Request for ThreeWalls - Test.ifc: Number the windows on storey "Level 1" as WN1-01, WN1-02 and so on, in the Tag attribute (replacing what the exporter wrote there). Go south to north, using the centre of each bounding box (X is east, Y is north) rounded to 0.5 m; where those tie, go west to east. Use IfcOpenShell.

First a look at what the model holds.

```python
import ifcopenshell
import ifcopenshell.util.element
import ifcopenshell.util.placement

model = ifcopenshell.open("ThreeWalls - Test.ifc")
print(model.schema)
storey = next(s for s in model.by_type("IfcBuildingStorey") if s.Name == "Level 1")
windows = [e for e in ifcopenshell.util.element.get_decomposition(storey) if e.is_a("IfcWindow")]
for e in sorted(windows, key=lambda e: e.id()):
    origin = ifcopenshell.util.placement.get_local_placement(e.ObjectPlacement)[:3, 3]
    print(e.id(), e.Tag, e.Name, origin.round(2) + 0.0, sep=" | ")
```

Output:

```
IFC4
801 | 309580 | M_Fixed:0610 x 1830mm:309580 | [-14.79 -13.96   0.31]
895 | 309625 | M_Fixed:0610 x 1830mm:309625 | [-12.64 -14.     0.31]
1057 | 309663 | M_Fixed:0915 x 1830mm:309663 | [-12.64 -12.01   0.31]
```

```python
import ifcopenshell
import ifcopenshell.geom
import ifcopenshell.util.element
import ifcopenshell.util.shape

model = ifcopenshell.open("ThreeWalls - Test.ifc")
settings = ifcopenshell.geom.settings()
settings.set("use-world-coords", True)


def centre(element):
    shape = ifcopenshell.geom.create_shape(settings, element)
    return ifcopenshell.util.shape.get_bbox_centroid(shape.geometry)


storey = next(s for s in model.by_type("IfcBuildingStorey") if s.Name == "Level 1")
windows = [e for e in ifcopenshell.util.element.get_decomposition(storey) if e.is_a("IfcWindow")]

# Insertion points can sit at a corner or the storey origin, so sort by the geometry (in metres).
centres = {e: centre(e) for e in windows}
windows.sort(key=lambda e: (round(centres[e][1] / 0.5), centres[e][0]))

for i, e in enumerate(windows, start=1):
    number = f"WN1-{i:02d}"
    e.Tag = number
    print(e.id(), number)

model.write("ThreeWalls - Test_updated.ifc")
```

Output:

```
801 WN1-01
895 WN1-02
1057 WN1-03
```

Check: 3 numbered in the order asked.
